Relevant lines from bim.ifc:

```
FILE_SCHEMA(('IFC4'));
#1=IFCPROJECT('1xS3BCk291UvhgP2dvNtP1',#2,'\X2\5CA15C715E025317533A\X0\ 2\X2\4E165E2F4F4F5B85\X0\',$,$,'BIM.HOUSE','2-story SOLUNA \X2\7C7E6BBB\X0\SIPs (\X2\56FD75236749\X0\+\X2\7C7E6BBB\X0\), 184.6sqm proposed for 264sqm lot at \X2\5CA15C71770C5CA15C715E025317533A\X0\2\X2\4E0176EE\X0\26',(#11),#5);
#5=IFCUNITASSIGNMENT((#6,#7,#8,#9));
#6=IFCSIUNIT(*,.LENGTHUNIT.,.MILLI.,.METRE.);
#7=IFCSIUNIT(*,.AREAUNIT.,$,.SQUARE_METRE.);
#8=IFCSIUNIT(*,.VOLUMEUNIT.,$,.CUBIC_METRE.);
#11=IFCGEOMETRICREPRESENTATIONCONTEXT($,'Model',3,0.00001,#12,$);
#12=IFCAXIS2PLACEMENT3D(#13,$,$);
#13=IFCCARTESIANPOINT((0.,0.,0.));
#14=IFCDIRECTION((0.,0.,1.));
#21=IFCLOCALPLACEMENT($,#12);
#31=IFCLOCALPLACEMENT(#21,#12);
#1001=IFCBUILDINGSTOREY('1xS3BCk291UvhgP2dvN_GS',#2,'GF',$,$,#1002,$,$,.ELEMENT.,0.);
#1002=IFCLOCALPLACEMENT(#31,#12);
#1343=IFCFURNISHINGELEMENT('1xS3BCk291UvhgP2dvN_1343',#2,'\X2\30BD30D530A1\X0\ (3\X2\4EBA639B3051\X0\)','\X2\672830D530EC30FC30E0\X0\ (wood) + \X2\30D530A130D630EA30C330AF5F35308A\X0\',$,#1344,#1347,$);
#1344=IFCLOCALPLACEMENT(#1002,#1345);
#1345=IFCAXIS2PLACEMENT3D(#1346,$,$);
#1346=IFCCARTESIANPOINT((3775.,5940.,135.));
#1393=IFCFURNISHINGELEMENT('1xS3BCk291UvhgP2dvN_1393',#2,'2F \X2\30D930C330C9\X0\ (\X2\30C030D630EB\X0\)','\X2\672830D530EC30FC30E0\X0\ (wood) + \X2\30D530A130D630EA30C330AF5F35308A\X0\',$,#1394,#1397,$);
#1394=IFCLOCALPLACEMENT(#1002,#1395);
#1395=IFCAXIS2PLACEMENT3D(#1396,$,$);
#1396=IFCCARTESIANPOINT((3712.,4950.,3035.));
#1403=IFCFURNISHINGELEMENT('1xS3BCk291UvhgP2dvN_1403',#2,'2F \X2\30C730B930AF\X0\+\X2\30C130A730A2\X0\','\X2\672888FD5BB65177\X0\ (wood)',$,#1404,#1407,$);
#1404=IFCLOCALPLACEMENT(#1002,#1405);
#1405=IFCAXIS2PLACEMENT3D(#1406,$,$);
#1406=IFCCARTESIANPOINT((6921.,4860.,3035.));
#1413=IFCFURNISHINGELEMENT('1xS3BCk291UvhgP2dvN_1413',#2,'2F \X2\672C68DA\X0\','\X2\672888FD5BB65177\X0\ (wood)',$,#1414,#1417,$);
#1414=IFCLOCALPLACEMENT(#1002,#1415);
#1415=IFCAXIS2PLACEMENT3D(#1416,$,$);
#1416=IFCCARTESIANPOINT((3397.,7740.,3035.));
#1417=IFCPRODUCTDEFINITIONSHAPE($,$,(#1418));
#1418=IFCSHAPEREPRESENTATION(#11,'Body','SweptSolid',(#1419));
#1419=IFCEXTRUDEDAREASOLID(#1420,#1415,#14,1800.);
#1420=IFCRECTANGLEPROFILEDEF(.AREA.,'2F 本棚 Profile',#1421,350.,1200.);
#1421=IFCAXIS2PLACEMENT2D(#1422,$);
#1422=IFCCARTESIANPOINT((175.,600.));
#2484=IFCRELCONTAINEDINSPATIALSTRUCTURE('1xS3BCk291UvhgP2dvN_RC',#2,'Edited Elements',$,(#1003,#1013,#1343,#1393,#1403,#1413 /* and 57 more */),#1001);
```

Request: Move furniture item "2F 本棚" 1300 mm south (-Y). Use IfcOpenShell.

```python
import ifcopenshell
import ifcopenshell.api.geometry
import ifcopenshell.util.placement
import ifcopenshell.util.unit

model = ifcopenshell.open("bim.ifc")
unit_scale = ifcopenshell.util.unit.calculate_unit_scale(model)

item = model.by_guid("1xS3BCk291UvhgP2dvN_1413")
matrix = ifcopenshell.util.placement.get_local_placement(item.ObjectPlacement)
matrix[1, 3] -= 1.3 / unit_scale
ifcopenshell.api.geometry.edit_object_placement(model, product=item, matrix=matrix, is_si=False)

print(ifcopenshell.util.placement.get_local_placement(item.ObjectPlacement).round(3) + 0.0)

model.write("bim_v2.ifc")
```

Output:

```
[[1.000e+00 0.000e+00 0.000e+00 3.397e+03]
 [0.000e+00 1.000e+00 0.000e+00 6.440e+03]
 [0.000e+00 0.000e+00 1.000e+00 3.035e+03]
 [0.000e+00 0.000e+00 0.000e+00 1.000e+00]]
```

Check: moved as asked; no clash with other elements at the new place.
